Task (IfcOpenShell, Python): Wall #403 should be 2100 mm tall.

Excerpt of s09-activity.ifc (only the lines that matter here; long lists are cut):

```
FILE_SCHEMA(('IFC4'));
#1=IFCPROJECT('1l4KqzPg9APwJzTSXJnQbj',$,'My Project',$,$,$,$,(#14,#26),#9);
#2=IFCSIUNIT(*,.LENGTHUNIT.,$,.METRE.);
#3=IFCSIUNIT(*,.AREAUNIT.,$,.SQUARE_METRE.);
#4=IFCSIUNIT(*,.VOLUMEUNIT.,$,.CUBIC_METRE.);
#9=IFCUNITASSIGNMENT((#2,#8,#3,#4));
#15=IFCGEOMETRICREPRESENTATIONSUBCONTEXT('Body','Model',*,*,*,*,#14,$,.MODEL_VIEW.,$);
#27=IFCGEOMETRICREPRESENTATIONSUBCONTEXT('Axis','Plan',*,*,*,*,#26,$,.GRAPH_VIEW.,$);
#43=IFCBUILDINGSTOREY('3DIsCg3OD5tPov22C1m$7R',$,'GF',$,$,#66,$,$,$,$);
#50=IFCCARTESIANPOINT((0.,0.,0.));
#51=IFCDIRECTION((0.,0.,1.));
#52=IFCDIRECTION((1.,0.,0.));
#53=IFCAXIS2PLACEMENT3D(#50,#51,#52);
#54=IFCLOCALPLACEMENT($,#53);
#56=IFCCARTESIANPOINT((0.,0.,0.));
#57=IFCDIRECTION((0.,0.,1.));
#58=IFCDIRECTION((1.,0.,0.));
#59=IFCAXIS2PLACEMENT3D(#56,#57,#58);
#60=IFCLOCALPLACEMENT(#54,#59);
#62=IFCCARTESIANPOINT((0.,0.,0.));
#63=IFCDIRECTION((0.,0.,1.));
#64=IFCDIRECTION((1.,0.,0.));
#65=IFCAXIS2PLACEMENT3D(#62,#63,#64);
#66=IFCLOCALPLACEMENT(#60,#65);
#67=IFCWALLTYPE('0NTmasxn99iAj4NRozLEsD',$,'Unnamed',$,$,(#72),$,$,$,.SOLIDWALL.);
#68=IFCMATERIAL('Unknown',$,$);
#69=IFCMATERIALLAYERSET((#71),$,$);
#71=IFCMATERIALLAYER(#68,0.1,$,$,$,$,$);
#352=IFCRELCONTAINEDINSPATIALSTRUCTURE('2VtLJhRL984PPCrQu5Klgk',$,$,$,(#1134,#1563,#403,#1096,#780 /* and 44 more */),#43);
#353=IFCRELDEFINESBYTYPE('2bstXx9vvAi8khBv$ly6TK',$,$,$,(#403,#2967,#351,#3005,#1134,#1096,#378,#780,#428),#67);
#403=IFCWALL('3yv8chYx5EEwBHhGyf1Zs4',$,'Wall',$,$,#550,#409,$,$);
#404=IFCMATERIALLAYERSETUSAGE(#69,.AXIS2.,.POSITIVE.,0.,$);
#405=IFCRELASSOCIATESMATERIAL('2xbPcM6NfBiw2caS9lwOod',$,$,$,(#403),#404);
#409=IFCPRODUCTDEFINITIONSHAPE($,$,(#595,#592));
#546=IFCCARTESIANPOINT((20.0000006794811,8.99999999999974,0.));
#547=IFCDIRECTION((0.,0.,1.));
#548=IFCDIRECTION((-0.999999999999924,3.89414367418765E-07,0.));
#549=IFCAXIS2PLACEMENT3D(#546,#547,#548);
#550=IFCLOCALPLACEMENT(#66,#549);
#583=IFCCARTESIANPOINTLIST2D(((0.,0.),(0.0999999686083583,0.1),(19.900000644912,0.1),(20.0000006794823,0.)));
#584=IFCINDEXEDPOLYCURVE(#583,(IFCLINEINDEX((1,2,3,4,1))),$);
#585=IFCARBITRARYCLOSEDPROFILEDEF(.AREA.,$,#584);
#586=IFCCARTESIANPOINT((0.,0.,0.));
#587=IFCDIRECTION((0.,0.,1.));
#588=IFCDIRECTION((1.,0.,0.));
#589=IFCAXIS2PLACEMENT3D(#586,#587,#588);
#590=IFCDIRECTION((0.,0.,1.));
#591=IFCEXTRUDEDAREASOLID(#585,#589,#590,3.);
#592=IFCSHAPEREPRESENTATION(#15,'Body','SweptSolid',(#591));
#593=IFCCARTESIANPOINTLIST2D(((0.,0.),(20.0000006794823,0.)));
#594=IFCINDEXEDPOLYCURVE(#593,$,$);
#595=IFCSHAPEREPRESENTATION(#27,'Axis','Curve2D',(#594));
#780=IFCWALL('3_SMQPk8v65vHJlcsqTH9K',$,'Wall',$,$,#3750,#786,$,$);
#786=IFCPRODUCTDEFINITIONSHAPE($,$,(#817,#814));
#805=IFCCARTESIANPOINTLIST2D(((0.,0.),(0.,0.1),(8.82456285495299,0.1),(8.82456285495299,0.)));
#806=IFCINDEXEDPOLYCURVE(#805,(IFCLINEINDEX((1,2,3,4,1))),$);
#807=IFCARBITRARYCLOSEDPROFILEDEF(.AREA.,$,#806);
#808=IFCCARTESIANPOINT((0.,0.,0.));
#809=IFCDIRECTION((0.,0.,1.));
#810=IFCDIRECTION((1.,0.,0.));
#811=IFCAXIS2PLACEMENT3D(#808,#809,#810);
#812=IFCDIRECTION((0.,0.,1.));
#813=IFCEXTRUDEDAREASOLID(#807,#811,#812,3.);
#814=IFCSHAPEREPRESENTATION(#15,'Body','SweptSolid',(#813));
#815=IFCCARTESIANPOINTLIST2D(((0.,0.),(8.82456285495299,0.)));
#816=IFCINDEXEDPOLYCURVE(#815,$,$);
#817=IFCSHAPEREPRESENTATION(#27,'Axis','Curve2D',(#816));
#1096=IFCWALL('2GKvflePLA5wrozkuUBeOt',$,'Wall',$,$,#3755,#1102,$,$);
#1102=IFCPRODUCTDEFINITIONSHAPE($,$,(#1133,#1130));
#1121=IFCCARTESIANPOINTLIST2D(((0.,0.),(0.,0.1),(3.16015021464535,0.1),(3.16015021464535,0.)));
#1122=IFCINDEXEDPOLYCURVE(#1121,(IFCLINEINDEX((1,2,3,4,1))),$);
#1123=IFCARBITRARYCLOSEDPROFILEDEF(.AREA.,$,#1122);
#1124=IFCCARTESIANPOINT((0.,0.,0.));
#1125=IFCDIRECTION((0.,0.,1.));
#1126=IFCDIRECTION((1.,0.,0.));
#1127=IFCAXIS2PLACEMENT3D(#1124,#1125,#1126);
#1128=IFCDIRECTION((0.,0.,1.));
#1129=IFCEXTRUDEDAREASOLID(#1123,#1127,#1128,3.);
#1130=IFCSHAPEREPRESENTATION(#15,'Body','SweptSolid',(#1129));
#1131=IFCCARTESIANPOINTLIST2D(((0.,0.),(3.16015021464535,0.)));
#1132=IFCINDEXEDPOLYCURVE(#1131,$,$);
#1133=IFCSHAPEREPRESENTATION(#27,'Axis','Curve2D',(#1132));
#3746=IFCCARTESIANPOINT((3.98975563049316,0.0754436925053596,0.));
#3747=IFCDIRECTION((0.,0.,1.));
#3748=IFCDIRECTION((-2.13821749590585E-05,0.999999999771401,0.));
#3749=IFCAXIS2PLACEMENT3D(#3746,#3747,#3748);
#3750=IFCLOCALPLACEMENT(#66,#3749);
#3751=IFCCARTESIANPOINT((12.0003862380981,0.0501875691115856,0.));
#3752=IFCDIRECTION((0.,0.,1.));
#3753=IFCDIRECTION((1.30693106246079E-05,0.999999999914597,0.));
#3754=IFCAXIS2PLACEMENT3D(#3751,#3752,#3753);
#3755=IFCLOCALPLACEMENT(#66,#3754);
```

```python
import ifcopenshell
import ifcopenshell.geom
import ifcopenshell.util.representation
import ifcopenshell.util.shape
import ifcopenshell.util.unit

model = ifcopenshell.open("s09-activity.ifc")
unit_scale = ifcopenshell.util.unit.calculate_unit_scale(model)
settings = ifcopenshell.geom.settings()


def volume(element):
    """Net volume in cubic metres, openings subtracted."""
    shape = ifcopenshell.geom.create_shape(settings, element)
    return ifcopenshell.util.shape.get_volume(shape.geometry)


wall = model.by_id(403)
before = volume(wall)

body = ifcopenshell.util.representation.get_representation(wall, "Model", "Body")
solid = body.Items[0]
old_height = solid.Depth
solid.Depth = 2.1 / unit_scale
after = volume(wall)

print(f"height {old_height:g} -> {solid.Depth:g}, volume {before:.3f} -> {after:.3f} m3")

model.write("s09-activity_rev.ifc")
```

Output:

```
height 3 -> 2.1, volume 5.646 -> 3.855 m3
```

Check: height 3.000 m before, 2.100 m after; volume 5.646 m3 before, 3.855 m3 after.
